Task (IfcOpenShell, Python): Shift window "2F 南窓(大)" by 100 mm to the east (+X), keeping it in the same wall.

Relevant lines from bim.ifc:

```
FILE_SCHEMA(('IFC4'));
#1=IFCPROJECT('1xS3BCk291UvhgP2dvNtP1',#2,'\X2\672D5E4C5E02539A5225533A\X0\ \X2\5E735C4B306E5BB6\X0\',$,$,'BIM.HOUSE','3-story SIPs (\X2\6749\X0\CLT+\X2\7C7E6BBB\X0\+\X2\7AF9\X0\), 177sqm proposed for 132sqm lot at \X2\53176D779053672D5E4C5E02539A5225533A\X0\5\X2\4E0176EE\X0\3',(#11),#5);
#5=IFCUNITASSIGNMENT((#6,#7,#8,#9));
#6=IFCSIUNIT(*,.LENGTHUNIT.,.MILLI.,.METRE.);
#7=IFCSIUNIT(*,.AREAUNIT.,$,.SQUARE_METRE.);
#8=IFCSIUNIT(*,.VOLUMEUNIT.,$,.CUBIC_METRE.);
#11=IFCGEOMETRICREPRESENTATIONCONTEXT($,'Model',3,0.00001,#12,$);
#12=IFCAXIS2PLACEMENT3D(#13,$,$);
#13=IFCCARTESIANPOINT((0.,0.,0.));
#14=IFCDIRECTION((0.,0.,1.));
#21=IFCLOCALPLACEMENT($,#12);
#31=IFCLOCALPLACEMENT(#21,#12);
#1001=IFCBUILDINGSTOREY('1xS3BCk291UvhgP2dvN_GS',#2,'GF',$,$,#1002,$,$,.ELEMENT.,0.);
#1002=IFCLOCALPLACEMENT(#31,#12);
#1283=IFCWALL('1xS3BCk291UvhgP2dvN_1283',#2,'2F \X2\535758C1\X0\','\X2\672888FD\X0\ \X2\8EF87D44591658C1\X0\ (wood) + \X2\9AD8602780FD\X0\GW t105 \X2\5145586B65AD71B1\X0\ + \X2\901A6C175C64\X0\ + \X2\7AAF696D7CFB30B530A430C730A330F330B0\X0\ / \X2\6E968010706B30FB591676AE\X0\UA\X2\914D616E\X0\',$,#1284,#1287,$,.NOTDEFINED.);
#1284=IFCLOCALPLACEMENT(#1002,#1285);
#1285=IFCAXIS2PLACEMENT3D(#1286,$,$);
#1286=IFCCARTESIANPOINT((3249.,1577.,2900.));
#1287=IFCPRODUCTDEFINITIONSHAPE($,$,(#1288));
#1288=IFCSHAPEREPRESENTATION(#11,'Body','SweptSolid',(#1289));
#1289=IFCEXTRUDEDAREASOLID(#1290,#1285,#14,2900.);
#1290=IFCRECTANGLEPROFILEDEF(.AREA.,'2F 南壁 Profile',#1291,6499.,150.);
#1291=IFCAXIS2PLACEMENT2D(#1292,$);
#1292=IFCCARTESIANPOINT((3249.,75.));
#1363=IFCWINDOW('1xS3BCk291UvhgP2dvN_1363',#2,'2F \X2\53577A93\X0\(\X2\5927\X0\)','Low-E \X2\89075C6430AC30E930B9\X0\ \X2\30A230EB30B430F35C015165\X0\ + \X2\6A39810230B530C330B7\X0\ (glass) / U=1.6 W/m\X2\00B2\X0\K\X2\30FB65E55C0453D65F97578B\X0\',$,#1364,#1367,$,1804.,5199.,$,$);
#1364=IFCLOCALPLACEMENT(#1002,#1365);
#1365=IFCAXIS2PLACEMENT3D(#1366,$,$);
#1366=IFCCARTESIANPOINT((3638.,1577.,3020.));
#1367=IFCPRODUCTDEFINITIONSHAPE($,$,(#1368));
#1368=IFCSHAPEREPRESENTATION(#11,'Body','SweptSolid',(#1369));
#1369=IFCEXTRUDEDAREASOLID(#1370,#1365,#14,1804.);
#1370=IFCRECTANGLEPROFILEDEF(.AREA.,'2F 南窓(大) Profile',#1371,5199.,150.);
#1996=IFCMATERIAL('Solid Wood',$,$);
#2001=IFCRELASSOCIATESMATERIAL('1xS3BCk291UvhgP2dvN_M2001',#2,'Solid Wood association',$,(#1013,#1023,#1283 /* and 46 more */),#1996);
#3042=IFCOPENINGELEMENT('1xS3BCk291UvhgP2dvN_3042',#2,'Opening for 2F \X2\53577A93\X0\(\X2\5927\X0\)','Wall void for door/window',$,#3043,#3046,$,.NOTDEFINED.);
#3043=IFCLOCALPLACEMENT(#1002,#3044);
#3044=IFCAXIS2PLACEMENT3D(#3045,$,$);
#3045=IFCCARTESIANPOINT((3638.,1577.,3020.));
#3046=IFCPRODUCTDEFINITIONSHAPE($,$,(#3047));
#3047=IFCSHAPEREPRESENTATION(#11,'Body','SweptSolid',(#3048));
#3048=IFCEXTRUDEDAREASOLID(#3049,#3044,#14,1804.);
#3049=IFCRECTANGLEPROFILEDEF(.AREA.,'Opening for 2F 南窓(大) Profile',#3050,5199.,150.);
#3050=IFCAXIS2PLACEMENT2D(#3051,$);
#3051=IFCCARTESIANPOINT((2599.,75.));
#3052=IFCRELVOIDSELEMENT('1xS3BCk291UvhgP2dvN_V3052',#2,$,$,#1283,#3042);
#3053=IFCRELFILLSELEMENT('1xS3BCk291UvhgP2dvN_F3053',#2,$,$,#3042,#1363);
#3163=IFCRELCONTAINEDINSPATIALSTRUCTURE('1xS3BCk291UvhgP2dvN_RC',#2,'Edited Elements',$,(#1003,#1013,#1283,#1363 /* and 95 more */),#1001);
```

```python
import ifcopenshell
import ifcopenshell.api.geometry
import ifcopenshell.util.placement
import ifcopenshell.util.unit

model = ifcopenshell.open("bim.ifc")
unit_scale = ifcopenshell.util.unit.calculate_unit_scale(model)

window = model.by_guid("1xS3BCk291UvhgP2dvN_1363")
opening = window.FillsVoids[0].RelatingOpeningElement
wall = opening.VoidsElements[0].RelatingBuildingElement

wall_matrix = ifcopenshell.util.placement.get_local_placement(wall.ObjectPlacement)
shift = wall_matrix[:3, 0] * 0.1 / unit_scale
before = ifcopenshell.util.placement.get_local_placement(window.ObjectPlacement)[:3, 3].copy()

# The window is not placed relative to its opening, so move both.
for product in (opening, window):
    matrix = ifcopenshell.util.placement.get_local_placement(product.ObjectPlacement)
    matrix[:3, 3] += shift
    ifcopenshell.api.geometry.edit_object_placement(model, product=product, matrix=matrix, is_si=False)

after = ifcopenshell.util.placement.get_local_placement(window.ObjectPlacement)[:3, 3]
print("window moved by", (after - before).round(3) + 0.0)

model.write("bim-out.ifc")
```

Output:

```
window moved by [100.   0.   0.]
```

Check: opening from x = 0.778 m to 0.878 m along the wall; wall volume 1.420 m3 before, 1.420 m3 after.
